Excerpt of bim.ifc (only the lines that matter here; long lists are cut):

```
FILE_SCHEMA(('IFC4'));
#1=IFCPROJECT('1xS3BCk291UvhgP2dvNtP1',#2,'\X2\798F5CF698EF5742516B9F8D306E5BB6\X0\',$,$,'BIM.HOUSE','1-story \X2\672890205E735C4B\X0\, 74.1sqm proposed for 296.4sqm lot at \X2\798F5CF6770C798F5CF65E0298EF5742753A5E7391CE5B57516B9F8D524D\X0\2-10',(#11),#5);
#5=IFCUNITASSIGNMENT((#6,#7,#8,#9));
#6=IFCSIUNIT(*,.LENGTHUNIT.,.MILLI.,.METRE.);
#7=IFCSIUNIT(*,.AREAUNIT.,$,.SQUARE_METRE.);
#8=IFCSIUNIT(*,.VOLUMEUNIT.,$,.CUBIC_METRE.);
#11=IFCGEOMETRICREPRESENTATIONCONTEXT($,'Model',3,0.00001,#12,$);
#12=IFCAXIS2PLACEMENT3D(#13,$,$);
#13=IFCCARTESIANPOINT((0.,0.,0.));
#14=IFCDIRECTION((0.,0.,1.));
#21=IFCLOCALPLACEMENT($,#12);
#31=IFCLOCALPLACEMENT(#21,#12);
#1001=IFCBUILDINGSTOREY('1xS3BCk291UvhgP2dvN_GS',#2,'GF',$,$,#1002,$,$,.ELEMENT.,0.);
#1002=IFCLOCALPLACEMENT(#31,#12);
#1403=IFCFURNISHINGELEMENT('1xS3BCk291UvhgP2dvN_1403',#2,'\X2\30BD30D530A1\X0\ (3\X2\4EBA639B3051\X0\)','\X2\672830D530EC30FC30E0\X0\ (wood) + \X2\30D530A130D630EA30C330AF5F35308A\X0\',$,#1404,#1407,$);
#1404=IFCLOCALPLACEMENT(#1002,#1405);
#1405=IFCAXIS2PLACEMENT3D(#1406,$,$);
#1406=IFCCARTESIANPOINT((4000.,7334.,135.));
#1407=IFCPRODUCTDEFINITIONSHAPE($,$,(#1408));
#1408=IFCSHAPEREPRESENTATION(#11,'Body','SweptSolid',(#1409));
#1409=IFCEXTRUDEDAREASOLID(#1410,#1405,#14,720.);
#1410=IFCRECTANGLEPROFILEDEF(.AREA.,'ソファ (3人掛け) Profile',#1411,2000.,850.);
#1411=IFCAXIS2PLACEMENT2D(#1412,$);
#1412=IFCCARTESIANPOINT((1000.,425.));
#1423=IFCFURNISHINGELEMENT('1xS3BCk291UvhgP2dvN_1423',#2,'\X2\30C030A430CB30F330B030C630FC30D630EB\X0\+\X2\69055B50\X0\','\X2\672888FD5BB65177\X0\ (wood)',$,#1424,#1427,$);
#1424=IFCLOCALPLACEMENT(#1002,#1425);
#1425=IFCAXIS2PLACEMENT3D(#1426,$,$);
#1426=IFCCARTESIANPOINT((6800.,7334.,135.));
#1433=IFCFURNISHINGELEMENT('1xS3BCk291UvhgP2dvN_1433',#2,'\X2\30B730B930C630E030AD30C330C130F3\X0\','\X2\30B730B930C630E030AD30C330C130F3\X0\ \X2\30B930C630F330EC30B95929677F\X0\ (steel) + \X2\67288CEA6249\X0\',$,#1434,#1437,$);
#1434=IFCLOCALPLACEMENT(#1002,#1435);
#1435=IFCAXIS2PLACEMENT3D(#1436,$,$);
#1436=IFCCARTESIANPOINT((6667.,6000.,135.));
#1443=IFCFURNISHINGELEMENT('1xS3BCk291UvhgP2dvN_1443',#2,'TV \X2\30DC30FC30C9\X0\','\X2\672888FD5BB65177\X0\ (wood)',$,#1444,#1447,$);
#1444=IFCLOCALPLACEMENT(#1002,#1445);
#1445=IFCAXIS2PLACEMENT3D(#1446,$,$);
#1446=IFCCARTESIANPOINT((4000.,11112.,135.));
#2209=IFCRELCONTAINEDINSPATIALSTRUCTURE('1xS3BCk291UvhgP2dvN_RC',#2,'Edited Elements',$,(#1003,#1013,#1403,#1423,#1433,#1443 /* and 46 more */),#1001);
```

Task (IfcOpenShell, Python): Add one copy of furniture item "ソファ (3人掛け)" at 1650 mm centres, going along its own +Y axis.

```python
import ifcopenshell
import ifcopenshell.api.geometry
import ifcopenshell.api.root
import ifcopenshell.util.element
import ifcopenshell.util.placement
import ifcopenshell.util.unit

model = ifcopenshell.open("bim.ifc")
unit_scale = ifcopenshell.util.unit.calculate_unit_scale(model)


def reuse_history(source, copy):
    """copy_class also copies each property set's owner history, people and application; keep the originals."""
    for rel in copy.IsDefinedBy:
        if rel.is_a("IfcRelDefinesByProperties") and (history := rel.RelatingPropertyDefinition.OwnerHistory):
            rel.RelatingPropertyDefinition.OwnerHistory = source.OwnerHistory
            ifcopenshell.util.element.remove_deep2(model, history)


source = model.by_guid("1xS3BCk291UvhgP2dvN_1403")
base = ifcopenshell.util.placement.get_local_placement(source.ObjectPlacement)
step = base[:3, 1] * 1.65 / unit_scale

for i in range(1, 2):
    copy = ifcopenshell.api.root.copy_class(model, product=source)
    copy.Representation = ifcopenshell.util.element.copy_deep(
        model, source.Representation, exclude=["IfcGeometricRepresentationContext", "IfcRepresentationMap"]
    )
    reuse_history(source, copy)
    matrix = base.copy()
    matrix[:3, 3] += i * step
    print("added at", matrix[:3, 3].round(3) + 0.0)
    ifcopenshell.api.geometry.edit_object_placement(model, product=copy, matrix=matrix, is_si=False)

model.write("bim-out.ifc")
```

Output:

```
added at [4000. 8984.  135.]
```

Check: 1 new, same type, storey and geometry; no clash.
